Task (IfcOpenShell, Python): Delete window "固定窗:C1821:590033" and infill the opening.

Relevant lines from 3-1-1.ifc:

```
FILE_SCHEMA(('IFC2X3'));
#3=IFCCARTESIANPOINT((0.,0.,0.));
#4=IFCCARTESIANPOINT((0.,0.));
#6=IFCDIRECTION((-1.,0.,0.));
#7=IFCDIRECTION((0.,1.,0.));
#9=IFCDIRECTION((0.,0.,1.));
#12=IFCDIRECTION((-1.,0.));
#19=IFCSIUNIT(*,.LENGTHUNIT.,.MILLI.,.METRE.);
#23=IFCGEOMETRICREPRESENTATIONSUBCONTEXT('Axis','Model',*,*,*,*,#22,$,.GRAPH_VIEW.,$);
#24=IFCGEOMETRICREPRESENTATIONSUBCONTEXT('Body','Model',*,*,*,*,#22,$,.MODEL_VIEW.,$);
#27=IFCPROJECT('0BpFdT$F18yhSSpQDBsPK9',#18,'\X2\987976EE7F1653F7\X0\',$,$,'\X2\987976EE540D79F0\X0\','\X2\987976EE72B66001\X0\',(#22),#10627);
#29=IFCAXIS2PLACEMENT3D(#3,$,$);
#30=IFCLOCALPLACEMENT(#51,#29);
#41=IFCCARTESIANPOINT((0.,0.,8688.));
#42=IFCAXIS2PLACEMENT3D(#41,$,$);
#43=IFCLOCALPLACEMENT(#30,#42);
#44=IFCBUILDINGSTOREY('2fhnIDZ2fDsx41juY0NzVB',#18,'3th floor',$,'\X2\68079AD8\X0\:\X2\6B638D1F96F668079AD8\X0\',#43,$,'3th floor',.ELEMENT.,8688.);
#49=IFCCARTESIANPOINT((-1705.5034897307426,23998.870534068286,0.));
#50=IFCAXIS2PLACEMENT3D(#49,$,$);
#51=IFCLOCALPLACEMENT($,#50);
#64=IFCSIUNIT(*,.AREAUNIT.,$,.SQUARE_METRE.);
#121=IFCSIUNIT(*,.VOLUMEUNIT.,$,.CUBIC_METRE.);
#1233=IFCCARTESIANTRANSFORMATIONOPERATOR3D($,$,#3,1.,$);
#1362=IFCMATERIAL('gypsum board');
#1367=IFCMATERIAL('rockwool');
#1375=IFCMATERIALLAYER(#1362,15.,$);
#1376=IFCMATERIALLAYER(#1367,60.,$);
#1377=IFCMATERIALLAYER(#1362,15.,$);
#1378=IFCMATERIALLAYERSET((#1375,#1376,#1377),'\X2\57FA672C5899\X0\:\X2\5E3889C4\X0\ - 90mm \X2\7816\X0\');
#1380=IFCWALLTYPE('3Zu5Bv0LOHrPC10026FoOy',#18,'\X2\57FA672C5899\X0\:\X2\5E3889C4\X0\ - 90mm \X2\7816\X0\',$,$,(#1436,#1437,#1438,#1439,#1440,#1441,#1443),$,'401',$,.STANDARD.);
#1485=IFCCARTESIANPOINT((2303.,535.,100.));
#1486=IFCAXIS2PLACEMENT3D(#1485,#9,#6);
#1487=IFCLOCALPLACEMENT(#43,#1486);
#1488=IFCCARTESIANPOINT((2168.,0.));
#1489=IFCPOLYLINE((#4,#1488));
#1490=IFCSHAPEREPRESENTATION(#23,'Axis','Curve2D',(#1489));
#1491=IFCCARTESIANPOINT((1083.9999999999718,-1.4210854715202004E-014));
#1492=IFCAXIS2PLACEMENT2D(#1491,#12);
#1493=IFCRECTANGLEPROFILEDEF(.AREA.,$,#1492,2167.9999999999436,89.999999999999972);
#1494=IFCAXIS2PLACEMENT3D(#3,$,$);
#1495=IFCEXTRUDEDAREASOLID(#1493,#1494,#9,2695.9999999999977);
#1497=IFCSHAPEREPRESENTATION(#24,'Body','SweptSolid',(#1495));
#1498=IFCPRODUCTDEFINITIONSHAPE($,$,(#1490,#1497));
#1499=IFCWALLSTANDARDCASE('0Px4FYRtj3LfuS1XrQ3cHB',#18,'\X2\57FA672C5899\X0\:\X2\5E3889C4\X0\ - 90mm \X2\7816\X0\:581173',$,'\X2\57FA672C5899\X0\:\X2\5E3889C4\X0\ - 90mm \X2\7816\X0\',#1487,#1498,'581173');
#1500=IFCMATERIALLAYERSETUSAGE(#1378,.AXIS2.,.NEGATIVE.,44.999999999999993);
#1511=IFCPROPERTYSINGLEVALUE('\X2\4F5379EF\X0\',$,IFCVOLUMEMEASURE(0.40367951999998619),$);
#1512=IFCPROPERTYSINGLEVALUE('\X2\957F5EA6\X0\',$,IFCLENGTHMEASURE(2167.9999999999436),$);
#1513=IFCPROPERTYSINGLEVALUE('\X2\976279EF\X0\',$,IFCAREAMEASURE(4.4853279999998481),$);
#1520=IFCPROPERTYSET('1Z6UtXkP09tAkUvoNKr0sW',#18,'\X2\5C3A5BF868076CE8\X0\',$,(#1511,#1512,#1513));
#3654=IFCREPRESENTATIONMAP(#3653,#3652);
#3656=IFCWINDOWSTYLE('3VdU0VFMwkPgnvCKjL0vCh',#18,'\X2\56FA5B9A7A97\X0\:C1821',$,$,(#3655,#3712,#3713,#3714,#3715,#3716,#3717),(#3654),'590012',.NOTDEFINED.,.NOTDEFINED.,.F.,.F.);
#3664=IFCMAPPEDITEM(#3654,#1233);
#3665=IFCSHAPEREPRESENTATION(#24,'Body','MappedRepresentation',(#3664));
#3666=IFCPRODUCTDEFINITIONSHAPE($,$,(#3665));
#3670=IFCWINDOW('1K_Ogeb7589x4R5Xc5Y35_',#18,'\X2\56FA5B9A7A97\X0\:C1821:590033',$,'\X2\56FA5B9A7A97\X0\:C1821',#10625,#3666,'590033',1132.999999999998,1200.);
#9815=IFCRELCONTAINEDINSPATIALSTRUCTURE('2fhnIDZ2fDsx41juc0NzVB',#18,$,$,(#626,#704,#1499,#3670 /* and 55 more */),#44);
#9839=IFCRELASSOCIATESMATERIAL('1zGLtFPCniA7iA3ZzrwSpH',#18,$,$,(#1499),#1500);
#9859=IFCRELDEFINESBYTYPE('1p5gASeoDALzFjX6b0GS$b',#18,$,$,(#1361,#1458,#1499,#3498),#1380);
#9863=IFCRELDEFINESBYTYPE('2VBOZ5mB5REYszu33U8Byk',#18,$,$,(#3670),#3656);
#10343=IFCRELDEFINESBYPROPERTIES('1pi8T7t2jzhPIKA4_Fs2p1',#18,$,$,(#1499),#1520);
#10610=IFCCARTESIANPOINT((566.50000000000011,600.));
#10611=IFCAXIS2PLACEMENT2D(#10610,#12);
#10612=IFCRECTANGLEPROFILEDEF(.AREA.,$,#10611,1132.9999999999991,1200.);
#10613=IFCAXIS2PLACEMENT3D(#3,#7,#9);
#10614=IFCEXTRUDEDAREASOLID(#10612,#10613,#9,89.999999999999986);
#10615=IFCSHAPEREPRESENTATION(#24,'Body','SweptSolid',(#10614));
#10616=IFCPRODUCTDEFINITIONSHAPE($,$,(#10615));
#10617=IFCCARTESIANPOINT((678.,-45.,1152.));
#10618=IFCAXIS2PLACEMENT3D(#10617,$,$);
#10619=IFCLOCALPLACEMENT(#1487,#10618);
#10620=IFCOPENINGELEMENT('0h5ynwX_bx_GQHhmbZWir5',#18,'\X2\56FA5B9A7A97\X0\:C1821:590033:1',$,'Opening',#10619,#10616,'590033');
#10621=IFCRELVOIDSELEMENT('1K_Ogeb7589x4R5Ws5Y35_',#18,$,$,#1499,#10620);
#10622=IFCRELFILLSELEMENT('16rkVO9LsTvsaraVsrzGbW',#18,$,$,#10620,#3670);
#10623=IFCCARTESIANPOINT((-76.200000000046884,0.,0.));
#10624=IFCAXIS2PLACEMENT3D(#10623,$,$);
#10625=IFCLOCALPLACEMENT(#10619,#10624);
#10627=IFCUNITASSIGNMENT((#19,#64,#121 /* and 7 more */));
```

```python
import ifcopenshell
import ifcopenshell.api.feature
import ifcopenshell.api.pset
import ifcopenshell.api.root
import ifcopenshell.geom
import ifcopenshell.util.element
import ifcopenshell.util.shape
import ifcopenshell.util.unit

model = ifcopenshell.open("3-1-1.ifc")
area_scale = ifcopenshell.util.unit.calculate_unit_scale(model, "AREAUNIT")
volume_scale = ifcopenshell.util.unit.calculate_unit_scale(model, "VOLUMEUNIT")
settings = ifcopenshell.geom.settings()


def volume(element):
    """Net volume in cubic metres, openings subtracted."""
    shape = ifcopenshell.geom.create_shape(settings, element)
    return ifcopenshell.util.shape.get_volume(shape.geometry)


window = model.by_guid("1K_Ogeb7589x4R5Xc5Y35_")
opening = window.FillsVoids[0].RelatingOpeningElement
wall = opening.VoidsElements[0].RelatingBuildingElement
before = volume(wall)

ifcopenshell.api.root.remove_product(model, product=window)
ifcopenshell.api.feature.remove_feature(model, feature=opening)

after = volume(wall)
thickness = 0.09  # wall thickness in metres

# Update the wall's stored quantities.
pset = model.by_id(ifcopenshell.util.element.get_pset(wall, "尺寸标注", should_inherit=False)["id"])
ifcopenshell.api.pset.edit_pset(model, pset=pset, properties={
    "体积": model.create_entity("IfcVolumeMeasure", after / volume_scale),
    "面积": model.create_entity("IfcAreaMeasure", after / thickness / area_scale),
})

print(f"wall volume {before:.3f} -> {after:.3f} m3")

model.write("3-1-1-out.ifc")
```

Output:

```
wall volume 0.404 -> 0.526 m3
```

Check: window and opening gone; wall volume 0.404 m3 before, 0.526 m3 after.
